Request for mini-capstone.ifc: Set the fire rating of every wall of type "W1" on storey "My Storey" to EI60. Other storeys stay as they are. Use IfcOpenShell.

First a look at what the model holds.

```python
import ifcopenshell
import ifcopenshell.util.element

model = ifcopenshell.open("mini-capstone.ifc")
print(model.schema)
storey = next(s for s in model.by_type("IfcBuildingStorey") if s.Name == "My Storey")
walls = [e for e in ifcopenshell.util.element.get_decomposition(storey) if e.is_a("IfcWall")]
seen = {}
for e in walls:
    element_type = ifcopenshell.util.element.get_type(e)
    key = (element_type.Name if element_type != e and element_type else None, ifcopenshell.util.element.get_pset(e, "Pset_WallCommon", "FireRating"))
    seen[key] = seen.get(key, 0) + 1
for (name, value), count in sorted(seen.items(), key=str):
    print(count, "x", name, "|", value)
```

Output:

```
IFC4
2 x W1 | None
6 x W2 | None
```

```python
import ifcopenshell
import ifcopenshell.api.pset
import ifcopenshell.util.element

model = ifcopenshell.open("mini-capstone.ifc")

storey = next(s for s in model.by_type("IfcBuildingStorey") if s.Name == "My Storey")
walls = [e for e in ifcopenshell.util.element.get_decomposition(storey) if e.is_a("IfcWall")]

count = 0
for e in walls:
    element_type = ifcopenshell.util.element.get_type(e)
    if element_type in (None, e) or element_type.Name != "W1":
        continue
    # add_pset returns the element's existing set when there is one.
    pset = ifcopenshell.api.pset.add_pset(model, product=e, name="Pset_WallCommon")
    ifcopenshell.api.pset.edit_pset(model, pset=pset, properties={"FireRating": "EI60"})
    count += 1

print(count, "walls updated")

model.write("mini-capstone_v2.ifc")
```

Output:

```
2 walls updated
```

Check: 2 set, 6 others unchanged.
